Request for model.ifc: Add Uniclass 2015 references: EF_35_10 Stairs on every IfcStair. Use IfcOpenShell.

First a look at what the model holds.

```python
import ifcopenshell

model = ifcopenshell.open("model.ifc")
print(model.schema)
print("classifications:", [c.Name for c in model.by_type("IfcClassification")])
for ifc_class in ("IfcDoor", "IfcRoof", "IfcStair", "IfcWall", "IfcWindow"):
    print(ifc_class, len(model.by_type(ifc_class)))
```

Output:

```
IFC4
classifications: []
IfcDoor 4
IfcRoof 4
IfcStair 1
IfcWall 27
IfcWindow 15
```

```python
import ifcopenshell
import ifcopenshell.api.classification

model = ifcopenshell.open("model.ifc")

system = ifcopenshell.api.classification.add_classification(model, classification="Uniclass 2015")

codes = {
    "IfcStair": ("EF_35_10", "Stairs"),
}
for ifc_class, (code, name) in codes.items():
    products = model.by_type(ifc_class)
    ifcopenshell.api.classification.add_reference(
        model, products=products, classification=system, identification=code, name=name
    )
    print(code, len(products))

model.write("model_v2.ifc")
```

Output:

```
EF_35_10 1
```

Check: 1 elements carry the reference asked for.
